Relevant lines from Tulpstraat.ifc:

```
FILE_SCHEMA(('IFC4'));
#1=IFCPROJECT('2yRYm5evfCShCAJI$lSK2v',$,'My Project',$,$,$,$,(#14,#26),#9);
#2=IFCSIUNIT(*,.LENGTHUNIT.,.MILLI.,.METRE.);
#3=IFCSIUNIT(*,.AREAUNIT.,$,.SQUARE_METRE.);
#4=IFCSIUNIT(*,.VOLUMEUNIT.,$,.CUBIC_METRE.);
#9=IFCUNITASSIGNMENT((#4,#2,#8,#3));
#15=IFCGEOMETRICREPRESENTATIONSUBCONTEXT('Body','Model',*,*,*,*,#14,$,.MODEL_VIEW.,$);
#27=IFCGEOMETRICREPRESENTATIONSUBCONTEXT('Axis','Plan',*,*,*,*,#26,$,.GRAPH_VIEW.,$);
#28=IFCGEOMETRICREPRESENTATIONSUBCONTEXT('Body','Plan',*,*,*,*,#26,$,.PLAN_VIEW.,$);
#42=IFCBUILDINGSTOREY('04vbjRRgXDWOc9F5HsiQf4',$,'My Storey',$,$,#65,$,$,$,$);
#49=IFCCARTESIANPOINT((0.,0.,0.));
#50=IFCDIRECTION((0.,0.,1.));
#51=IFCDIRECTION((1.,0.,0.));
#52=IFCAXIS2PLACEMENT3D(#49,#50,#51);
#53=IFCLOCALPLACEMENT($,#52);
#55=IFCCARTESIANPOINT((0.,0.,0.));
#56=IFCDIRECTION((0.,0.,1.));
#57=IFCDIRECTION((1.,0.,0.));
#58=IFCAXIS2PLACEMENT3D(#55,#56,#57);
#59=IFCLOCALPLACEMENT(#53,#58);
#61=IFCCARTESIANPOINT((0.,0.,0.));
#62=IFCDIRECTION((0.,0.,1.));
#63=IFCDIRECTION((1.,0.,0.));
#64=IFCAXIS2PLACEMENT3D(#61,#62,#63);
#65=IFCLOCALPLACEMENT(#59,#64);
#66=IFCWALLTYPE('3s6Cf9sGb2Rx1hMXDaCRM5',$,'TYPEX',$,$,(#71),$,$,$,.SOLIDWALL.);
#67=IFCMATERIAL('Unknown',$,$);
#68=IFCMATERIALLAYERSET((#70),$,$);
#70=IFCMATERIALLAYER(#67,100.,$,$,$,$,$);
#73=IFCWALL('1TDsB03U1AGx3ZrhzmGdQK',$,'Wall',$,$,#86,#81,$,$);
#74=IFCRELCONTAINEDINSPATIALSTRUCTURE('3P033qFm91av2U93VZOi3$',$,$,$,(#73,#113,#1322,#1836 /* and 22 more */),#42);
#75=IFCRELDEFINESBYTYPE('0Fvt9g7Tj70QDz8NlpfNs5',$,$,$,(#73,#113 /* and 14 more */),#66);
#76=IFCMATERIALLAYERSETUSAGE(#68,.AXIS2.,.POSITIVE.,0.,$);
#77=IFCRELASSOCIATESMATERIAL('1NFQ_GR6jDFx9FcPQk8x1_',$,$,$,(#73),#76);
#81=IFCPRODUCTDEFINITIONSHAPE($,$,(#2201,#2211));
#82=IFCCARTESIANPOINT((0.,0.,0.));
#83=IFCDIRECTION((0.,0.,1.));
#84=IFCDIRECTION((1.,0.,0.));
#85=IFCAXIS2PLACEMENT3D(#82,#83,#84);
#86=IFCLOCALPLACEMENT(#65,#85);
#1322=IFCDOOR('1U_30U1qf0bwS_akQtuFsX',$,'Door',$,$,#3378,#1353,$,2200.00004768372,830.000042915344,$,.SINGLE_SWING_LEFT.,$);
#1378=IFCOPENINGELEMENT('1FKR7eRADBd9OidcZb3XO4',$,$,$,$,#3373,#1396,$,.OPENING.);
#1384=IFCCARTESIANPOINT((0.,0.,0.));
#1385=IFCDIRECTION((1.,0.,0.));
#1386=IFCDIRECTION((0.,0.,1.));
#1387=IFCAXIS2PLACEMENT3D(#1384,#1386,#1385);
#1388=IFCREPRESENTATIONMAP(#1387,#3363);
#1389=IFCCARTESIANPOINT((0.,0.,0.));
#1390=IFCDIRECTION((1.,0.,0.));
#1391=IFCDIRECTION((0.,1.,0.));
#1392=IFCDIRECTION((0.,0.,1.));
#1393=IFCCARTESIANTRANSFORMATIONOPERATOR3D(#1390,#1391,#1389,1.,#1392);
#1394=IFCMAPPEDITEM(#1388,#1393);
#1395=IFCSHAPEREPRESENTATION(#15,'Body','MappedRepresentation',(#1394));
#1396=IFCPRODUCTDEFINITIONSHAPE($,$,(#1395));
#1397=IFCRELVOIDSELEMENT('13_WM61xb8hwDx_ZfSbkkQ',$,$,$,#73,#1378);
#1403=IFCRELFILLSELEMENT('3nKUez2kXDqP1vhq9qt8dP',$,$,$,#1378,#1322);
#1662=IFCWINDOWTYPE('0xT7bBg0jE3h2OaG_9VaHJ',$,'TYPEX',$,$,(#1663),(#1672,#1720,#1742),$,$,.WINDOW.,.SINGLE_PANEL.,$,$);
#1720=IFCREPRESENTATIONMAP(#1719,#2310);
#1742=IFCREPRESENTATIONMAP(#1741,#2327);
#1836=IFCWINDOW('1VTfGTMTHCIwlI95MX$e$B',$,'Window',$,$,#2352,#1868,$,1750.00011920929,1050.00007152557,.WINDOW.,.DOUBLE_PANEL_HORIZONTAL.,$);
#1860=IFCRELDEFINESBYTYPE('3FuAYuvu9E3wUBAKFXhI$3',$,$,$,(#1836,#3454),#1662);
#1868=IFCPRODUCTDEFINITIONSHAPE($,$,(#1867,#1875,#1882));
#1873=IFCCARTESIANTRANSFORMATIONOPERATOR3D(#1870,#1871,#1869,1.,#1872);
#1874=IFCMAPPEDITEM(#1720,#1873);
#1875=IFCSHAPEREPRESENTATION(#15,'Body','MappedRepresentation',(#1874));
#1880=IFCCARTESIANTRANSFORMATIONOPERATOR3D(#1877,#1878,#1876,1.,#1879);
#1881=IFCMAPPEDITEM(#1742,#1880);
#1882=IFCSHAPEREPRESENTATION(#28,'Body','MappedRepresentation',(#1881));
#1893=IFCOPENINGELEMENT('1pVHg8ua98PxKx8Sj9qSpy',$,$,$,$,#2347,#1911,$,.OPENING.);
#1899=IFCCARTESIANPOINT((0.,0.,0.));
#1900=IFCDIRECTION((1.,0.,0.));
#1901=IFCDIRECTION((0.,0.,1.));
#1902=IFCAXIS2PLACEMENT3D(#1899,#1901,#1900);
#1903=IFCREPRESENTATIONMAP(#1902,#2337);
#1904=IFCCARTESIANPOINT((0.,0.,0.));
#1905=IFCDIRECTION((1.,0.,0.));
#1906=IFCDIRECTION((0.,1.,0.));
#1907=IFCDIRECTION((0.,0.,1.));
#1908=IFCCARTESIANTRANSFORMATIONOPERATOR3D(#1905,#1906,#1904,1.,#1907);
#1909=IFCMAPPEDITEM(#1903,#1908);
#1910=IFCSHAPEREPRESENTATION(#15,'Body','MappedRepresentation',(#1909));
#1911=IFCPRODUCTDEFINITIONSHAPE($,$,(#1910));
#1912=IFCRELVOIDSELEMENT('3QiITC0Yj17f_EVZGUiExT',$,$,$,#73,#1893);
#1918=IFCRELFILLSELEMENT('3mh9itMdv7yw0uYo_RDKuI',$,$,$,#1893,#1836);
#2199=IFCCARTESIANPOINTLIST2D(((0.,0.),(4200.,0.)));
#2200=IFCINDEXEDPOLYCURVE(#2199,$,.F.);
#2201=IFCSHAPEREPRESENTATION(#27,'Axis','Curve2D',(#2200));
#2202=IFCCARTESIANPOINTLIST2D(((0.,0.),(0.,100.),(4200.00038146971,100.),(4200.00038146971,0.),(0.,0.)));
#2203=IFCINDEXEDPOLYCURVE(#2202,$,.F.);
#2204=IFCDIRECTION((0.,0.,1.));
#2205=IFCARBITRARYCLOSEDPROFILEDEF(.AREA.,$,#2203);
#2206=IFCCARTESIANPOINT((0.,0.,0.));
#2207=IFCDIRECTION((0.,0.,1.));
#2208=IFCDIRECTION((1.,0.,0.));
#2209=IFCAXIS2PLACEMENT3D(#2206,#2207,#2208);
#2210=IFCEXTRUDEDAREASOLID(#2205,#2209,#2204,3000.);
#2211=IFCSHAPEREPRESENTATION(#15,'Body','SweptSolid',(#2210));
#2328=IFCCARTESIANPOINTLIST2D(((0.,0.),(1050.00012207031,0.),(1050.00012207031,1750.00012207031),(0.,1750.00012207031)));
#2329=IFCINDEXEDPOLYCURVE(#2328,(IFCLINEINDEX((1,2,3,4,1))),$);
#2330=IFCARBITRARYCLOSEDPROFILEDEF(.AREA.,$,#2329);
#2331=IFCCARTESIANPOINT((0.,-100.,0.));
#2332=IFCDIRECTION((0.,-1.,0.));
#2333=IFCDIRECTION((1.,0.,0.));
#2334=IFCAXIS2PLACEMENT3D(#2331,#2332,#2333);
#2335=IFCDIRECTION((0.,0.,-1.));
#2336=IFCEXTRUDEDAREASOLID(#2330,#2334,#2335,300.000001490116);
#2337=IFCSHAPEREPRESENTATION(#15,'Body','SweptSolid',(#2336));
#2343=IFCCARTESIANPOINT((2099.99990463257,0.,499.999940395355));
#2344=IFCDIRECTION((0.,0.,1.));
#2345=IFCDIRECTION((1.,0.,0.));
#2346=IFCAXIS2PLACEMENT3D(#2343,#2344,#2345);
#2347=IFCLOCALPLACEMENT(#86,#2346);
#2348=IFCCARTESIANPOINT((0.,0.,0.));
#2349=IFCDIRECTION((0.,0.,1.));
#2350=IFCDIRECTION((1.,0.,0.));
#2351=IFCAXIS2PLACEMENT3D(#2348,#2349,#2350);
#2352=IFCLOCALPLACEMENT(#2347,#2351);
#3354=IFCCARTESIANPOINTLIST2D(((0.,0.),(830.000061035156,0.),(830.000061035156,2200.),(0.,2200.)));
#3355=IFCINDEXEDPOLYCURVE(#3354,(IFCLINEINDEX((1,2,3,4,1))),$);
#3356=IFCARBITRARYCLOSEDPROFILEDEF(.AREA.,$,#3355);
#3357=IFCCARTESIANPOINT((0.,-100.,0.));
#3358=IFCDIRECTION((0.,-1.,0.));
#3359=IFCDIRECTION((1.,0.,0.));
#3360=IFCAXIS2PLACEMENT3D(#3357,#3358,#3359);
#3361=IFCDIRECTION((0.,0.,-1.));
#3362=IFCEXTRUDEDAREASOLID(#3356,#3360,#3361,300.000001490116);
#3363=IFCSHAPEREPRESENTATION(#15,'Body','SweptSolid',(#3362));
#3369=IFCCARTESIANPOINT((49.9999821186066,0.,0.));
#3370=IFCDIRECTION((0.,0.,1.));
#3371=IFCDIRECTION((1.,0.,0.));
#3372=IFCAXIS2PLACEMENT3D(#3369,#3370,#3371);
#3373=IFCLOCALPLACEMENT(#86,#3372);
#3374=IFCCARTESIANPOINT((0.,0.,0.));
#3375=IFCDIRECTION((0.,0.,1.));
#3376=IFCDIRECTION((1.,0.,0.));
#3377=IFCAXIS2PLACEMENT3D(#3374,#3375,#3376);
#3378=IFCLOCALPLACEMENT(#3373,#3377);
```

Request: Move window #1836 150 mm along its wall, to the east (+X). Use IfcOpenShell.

```python
import ifcopenshell
import ifcopenshell.api.geometry
import ifcopenshell.util.placement
import ifcopenshell.util.unit

model = ifcopenshell.open("Tulpstraat.ifc")
unit_scale = ifcopenshell.util.unit.calculate_unit_scale(model)

window = model.by_guid("1VTfGTMTHCIwlI95MX$e$B")
opening = window.FillsVoids[0].RelatingOpeningElement
wall = opening.VoidsElements[0].RelatingBuildingElement

wall_matrix = ifcopenshell.util.placement.get_local_placement(wall.ObjectPlacement)
shift = wall_matrix[:3, 0] * 0.15 / unit_scale
before = ifcopenshell.util.placement.get_local_placement(window.ObjectPlacement)[:3, 3].copy()

# The window is placed relative to its opening, so it follows when the opening moves.
matrix = ifcopenshell.util.placement.get_local_placement(opening.ObjectPlacement)
matrix[:3, 3] += shift
ifcopenshell.api.geometry.edit_object_placement(
    model, product=opening, matrix=matrix, is_si=False, should_transform_children=True
)

after = ifcopenshell.util.placement.get_local_placement(window.ObjectPlacement)[:3, 3]
print("window moved by", (after - before).round(3) + 0.0)

model.write("Tulpstraat-out.ifc")
```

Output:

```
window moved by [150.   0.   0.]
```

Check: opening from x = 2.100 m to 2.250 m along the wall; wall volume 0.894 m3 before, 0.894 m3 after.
